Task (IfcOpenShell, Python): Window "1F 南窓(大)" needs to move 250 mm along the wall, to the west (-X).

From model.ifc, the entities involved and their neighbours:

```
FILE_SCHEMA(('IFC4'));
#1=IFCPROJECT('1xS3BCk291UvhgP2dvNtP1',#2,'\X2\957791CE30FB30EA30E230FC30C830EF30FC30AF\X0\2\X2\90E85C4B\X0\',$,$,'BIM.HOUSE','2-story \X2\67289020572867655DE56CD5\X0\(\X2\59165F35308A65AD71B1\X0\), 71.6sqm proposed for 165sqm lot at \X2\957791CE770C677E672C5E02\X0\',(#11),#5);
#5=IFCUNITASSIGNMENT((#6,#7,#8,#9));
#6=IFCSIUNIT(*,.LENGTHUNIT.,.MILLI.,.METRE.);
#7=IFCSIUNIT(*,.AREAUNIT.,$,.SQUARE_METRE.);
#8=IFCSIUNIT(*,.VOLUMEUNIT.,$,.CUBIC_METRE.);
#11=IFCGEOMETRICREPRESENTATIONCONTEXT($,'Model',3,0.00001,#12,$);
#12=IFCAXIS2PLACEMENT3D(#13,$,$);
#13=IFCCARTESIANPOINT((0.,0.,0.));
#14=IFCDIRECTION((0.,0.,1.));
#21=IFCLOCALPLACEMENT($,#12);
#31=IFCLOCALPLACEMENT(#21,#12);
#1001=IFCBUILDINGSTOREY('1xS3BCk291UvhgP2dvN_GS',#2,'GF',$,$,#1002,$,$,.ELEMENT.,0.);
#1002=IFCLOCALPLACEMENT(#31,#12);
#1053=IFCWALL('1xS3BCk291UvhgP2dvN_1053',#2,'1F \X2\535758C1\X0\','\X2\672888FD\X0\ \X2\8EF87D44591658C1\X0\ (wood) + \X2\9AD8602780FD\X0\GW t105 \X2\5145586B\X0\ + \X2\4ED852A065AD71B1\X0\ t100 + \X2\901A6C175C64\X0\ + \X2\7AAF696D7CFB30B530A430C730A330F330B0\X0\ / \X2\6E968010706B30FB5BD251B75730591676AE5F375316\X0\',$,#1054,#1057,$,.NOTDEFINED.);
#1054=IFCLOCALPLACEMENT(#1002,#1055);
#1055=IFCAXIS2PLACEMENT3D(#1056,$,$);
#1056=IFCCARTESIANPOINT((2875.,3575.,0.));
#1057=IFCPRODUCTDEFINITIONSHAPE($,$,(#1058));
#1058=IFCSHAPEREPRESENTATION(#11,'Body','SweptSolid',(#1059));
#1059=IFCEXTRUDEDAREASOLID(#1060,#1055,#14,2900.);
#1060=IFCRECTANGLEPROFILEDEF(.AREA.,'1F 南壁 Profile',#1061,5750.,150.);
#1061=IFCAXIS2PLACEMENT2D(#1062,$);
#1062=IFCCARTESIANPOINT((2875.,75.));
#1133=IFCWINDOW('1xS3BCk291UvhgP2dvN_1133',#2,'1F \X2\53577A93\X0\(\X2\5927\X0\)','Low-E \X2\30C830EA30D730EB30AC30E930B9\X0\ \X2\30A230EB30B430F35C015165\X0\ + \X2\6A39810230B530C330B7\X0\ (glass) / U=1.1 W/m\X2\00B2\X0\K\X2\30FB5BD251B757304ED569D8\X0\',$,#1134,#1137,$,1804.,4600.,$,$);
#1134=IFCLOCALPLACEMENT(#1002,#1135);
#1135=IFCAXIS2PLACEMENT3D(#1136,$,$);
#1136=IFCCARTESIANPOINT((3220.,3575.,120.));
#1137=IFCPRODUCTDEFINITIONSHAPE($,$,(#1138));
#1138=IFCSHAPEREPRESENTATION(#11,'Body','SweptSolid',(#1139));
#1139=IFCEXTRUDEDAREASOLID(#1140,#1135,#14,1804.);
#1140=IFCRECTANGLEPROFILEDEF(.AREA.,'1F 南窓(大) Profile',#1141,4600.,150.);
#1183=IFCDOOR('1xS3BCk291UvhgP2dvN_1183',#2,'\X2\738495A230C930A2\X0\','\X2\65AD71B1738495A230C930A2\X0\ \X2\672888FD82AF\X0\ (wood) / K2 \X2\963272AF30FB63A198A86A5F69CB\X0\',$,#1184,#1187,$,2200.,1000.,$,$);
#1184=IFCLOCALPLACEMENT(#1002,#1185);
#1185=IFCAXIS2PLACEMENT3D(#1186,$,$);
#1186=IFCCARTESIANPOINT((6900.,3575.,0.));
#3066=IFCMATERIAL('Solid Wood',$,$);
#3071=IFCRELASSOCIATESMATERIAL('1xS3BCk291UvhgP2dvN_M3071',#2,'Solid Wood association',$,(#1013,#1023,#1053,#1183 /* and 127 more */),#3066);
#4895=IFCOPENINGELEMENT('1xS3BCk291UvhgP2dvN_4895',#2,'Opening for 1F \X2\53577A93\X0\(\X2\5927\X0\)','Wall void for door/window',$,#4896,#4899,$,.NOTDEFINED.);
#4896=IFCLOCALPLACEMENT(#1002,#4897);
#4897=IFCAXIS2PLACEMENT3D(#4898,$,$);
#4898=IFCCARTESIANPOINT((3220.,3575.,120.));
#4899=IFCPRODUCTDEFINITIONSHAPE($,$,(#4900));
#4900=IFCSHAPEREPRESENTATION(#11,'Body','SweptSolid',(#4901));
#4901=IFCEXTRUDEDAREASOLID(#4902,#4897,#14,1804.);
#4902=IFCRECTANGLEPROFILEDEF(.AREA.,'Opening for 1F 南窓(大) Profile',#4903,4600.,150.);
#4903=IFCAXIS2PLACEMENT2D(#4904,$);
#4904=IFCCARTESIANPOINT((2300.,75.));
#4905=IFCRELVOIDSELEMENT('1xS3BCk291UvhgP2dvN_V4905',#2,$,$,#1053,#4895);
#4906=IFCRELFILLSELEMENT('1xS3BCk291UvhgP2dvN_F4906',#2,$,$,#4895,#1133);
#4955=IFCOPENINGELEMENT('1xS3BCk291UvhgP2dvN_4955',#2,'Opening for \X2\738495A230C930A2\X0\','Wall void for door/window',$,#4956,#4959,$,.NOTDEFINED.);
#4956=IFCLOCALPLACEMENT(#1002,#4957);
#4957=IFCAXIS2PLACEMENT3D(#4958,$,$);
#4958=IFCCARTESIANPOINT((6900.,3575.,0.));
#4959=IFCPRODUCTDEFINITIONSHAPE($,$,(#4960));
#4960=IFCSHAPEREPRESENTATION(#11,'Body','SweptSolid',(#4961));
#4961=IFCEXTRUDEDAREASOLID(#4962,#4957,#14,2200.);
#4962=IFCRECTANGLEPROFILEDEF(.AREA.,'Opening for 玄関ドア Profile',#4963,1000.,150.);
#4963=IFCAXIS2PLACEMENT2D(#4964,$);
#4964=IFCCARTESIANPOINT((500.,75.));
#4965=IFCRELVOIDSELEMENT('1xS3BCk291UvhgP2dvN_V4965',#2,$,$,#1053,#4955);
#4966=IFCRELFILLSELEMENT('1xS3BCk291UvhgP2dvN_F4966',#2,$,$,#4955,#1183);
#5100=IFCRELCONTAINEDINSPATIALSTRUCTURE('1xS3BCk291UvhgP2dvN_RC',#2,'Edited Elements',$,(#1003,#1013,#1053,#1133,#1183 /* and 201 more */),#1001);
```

```python
import ifcopenshell
import ifcopenshell.api.geometry
import ifcopenshell.util.placement
import ifcopenshell.util.unit

model = ifcopenshell.open("model.ifc")
unit_scale = ifcopenshell.util.unit.calculate_unit_scale(model)

window = model.by_id(1133)
opening = window.FillsVoids[0].RelatingOpeningElement
wall = opening.VoidsElements[0].RelatingBuildingElement

wall_matrix = ifcopenshell.util.placement.get_local_placement(wall.ObjectPlacement)
shift = wall_matrix[:3, 0] * -0.25 / unit_scale
before = ifcopenshell.util.placement.get_local_placement(window.ObjectPlacement)[:3, 3].copy()

# The window is not placed relative to its opening, so move both.
for product in (opening, window):
    matrix = ifcopenshell.util.placement.get_local_placement(product.ObjectPlacement)
    matrix[:3, 3] += shift
    ifcopenshell.api.geometry.edit_object_placement(model, product=product, matrix=matrix, is_si=False)

after = ifcopenshell.util.placement.get_local_placement(window.ObjectPlacement)[:3, 3]
print("window moved by", (after - before).round(3) + 0.0)

model.write("model_edited.ifc")
```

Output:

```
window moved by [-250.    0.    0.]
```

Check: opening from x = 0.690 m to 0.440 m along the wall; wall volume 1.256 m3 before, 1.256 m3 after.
